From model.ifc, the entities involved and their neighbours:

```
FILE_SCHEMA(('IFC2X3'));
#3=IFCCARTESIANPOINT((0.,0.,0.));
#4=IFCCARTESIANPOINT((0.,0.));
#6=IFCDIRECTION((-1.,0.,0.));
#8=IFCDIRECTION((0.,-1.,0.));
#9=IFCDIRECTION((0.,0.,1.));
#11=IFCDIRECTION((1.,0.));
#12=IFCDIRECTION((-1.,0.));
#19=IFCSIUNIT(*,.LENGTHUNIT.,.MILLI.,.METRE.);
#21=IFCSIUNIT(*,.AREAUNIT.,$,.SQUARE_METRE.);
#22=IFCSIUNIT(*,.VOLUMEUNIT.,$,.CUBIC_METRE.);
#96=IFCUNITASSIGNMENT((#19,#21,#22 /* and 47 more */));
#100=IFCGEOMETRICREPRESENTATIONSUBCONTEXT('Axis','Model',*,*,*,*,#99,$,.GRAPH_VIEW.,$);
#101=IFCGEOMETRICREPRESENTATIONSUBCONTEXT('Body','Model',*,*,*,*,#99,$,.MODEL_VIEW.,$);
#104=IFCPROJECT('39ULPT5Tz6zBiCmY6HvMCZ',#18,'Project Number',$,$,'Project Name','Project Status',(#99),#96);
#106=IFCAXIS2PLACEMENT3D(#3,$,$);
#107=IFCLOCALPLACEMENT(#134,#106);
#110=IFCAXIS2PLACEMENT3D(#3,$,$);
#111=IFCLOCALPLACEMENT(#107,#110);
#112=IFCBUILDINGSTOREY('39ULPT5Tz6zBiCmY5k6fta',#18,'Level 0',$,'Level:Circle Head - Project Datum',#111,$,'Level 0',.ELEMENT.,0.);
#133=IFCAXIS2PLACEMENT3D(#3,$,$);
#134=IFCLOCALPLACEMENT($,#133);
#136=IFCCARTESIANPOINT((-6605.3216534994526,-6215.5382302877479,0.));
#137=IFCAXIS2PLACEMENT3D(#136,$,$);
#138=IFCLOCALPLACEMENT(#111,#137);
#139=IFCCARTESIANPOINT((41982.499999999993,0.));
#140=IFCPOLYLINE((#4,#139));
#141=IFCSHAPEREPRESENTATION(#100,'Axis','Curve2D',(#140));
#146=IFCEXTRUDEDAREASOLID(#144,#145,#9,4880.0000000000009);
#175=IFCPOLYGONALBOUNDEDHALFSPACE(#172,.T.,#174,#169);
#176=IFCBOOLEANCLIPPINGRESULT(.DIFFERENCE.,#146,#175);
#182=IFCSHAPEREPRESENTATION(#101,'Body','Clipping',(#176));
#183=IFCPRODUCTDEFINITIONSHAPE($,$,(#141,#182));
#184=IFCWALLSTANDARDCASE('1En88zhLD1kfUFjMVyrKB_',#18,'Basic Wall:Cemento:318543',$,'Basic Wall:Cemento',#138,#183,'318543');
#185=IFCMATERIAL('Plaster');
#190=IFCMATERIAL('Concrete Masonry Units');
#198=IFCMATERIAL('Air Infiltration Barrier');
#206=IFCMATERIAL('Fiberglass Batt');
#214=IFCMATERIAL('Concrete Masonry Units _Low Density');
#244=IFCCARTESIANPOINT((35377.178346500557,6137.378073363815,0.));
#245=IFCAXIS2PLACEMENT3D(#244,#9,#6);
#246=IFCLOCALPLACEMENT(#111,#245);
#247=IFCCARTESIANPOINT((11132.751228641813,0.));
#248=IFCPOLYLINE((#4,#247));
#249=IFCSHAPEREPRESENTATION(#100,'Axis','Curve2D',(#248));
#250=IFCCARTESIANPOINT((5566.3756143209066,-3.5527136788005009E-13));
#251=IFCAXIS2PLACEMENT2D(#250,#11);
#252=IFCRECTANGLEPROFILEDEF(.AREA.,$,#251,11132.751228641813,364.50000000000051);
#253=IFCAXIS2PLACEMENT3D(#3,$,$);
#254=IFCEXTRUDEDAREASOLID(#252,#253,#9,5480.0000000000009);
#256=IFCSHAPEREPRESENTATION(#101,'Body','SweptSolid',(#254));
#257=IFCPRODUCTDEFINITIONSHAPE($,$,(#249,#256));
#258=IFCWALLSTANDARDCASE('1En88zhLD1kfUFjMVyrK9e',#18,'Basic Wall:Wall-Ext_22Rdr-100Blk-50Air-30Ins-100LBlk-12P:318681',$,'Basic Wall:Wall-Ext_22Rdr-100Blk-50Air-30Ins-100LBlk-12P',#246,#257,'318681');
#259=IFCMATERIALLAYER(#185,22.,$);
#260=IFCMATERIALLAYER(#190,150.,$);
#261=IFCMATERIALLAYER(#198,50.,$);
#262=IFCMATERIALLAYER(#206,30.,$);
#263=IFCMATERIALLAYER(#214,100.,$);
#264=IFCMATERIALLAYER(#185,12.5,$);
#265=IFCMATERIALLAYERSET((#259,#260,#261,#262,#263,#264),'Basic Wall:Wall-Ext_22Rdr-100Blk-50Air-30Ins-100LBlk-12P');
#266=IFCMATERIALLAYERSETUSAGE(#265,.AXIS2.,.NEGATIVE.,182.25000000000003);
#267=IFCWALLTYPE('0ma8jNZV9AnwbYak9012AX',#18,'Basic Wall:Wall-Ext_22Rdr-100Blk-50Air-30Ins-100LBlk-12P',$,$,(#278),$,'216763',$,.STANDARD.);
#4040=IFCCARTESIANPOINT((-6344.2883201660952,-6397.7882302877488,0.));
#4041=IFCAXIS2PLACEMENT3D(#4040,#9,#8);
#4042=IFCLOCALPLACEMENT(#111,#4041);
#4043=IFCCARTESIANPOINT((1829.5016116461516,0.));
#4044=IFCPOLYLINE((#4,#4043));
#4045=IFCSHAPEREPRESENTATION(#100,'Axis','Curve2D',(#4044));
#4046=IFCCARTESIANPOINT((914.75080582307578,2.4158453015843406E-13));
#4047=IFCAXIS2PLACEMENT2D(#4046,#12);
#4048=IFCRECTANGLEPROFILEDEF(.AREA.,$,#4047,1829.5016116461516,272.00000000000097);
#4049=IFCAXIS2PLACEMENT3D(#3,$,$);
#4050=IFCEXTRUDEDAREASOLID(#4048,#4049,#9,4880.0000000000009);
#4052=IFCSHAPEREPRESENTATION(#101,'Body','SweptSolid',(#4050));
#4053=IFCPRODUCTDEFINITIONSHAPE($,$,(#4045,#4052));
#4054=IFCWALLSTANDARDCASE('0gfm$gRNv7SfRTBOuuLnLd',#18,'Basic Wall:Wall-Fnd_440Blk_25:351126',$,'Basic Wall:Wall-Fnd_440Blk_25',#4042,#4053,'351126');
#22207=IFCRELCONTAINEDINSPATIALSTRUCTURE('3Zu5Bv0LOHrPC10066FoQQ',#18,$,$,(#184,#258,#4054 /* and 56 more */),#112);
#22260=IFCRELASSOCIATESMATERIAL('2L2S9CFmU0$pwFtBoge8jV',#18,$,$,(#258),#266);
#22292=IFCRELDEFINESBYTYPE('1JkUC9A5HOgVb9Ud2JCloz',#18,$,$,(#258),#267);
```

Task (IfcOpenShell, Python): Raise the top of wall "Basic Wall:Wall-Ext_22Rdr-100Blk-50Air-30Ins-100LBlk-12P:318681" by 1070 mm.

```python
import ifcopenshell
import ifcopenshell.geom
import ifcopenshell.util.representation
import ifcopenshell.util.shape
import ifcopenshell.util.unit

model = ifcopenshell.open("model.ifc")
unit_scale = ifcopenshell.util.unit.calculate_unit_scale(model)
settings = ifcopenshell.geom.settings()


def volume(element):
    """Net volume in cubic metres, openings subtracted."""
    shape = ifcopenshell.geom.create_shape(settings, element)
    return ifcopenshell.util.shape.get_volume(shape.geometry)


wall = model.by_id(258)
before = volume(wall)

body = ifcopenshell.util.representation.get_representation(wall, "Model", "Body")
solid = body.Items[0]
old_height = solid.Depth
solid.Depth += 1.07 / unit_scale
after = volume(wall)

print(f"height {old_height:g} -> {solid.Depth:g}, volume {before:.3f} -> {after:.3f} m3")

model.write("model_rev.ifc")
```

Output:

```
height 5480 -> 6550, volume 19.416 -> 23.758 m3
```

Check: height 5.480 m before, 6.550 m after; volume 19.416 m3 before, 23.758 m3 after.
